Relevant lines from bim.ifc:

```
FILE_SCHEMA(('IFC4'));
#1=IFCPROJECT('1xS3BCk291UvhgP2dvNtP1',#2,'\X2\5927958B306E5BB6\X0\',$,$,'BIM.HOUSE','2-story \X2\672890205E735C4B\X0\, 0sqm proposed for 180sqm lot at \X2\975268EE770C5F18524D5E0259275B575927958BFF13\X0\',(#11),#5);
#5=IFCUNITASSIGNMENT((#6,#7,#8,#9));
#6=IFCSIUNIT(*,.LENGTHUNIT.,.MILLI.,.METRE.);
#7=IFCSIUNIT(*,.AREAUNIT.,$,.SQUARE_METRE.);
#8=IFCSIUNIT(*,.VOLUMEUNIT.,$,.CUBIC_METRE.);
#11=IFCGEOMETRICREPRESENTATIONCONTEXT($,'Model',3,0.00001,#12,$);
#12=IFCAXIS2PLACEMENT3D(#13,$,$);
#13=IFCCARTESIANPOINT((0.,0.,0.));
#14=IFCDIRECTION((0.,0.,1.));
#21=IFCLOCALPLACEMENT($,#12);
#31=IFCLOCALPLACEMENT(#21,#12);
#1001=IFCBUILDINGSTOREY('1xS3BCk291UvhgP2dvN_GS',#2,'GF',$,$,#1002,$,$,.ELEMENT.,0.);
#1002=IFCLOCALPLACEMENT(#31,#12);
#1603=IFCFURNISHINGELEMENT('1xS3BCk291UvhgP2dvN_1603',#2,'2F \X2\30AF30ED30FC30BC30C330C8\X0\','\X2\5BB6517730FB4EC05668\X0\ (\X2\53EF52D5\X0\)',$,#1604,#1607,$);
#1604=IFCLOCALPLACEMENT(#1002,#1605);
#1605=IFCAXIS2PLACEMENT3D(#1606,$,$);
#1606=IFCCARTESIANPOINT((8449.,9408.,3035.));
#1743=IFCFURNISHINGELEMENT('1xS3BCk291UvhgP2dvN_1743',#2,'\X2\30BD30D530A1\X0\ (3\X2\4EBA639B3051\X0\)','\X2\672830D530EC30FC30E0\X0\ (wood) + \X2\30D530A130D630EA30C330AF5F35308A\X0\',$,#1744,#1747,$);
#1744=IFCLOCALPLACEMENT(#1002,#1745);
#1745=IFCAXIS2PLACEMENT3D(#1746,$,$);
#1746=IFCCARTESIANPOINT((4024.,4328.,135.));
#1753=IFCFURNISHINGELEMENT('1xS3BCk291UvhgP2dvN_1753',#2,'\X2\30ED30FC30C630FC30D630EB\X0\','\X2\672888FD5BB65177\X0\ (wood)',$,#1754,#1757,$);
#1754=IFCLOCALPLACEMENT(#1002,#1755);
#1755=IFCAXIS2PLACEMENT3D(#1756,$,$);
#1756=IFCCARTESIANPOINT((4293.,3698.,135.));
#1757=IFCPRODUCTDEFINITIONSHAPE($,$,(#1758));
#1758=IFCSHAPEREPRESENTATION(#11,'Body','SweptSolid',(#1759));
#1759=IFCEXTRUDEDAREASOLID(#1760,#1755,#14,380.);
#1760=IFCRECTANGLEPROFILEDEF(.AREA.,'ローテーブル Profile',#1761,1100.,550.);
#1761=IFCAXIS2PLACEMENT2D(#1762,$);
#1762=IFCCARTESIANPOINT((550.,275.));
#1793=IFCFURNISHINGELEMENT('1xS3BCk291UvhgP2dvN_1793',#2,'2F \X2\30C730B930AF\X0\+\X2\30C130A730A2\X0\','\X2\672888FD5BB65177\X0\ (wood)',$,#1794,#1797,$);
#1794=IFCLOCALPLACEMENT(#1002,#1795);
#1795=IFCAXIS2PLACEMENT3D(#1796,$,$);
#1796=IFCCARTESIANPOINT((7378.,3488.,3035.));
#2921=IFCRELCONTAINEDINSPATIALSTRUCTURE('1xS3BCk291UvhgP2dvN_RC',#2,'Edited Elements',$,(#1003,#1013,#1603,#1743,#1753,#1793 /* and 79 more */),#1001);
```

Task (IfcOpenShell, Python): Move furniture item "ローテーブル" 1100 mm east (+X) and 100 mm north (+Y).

```python
import ifcopenshell
import ifcopenshell.api.geometry
import ifcopenshell.util.placement
import ifcopenshell.util.unit

model = ifcopenshell.open("bim.ifc")
unit_scale = ifcopenshell.util.unit.calculate_unit_scale(model)

item = model.by_guid("1xS3BCk291UvhgP2dvN_1753")
matrix = ifcopenshell.util.placement.get_local_placement(item.ObjectPlacement)
matrix[0, 3] += 1.1 / unit_scale
matrix[1, 3] += 0.1 / unit_scale
ifcopenshell.api.geometry.edit_object_placement(model, product=item, matrix=matrix, is_si=False)

print(ifcopenshell.util.placement.get_local_placement(item.ObjectPlacement).round(3) + 0.0)

model.write("bim_rev.ifc")
```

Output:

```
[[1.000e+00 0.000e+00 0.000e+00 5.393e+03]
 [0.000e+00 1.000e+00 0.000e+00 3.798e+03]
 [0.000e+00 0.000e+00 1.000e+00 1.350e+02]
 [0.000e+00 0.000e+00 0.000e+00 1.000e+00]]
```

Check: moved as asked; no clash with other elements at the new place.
